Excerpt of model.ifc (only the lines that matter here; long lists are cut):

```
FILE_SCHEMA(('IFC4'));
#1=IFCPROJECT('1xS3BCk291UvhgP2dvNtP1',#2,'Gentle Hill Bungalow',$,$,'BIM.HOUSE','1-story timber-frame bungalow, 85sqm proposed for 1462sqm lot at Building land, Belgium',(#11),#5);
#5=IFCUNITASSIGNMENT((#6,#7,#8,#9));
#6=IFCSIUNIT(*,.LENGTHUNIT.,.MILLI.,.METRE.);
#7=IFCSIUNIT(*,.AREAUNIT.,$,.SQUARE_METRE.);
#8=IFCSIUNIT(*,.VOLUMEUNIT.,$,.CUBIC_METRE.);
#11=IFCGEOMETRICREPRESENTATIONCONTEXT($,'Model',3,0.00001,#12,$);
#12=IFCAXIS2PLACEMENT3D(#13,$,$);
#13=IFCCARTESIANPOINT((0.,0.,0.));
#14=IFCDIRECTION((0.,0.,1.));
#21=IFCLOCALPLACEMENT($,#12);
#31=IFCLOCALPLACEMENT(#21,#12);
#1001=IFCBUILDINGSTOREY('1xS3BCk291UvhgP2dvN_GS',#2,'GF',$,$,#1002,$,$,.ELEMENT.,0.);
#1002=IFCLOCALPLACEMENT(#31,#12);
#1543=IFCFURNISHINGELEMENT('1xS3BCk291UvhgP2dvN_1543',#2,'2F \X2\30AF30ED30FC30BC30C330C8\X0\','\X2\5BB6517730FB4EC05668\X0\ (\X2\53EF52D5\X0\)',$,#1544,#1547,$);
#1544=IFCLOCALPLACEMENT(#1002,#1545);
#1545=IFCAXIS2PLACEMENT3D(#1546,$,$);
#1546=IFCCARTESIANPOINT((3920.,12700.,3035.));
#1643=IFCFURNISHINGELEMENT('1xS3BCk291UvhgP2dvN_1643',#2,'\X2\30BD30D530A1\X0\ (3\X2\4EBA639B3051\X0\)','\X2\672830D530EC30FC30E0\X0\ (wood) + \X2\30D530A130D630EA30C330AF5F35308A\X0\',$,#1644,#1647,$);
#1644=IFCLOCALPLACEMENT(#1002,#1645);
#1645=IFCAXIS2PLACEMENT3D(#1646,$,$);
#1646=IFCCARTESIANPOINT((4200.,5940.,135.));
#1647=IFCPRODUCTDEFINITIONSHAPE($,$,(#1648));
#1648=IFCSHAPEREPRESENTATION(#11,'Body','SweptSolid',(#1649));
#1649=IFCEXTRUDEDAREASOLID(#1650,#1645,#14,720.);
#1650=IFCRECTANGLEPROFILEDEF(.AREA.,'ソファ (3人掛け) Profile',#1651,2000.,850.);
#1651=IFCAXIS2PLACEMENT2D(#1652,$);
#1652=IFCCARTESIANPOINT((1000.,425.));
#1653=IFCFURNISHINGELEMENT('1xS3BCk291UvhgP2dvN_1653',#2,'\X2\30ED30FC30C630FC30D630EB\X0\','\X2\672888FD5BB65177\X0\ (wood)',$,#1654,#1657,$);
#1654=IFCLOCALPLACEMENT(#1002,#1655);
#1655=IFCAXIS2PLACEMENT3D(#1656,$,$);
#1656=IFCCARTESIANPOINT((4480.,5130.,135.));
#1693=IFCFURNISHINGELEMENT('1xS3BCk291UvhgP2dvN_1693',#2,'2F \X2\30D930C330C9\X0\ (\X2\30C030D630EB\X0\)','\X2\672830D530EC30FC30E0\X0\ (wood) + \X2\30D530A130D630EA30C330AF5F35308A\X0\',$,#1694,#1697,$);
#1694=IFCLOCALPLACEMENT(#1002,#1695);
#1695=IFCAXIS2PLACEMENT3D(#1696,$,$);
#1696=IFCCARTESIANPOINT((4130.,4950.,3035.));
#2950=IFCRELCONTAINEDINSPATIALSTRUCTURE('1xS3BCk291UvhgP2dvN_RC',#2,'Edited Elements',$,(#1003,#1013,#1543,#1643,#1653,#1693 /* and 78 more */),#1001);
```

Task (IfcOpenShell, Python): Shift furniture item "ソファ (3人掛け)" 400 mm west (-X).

```python
import ifcopenshell
import ifcopenshell.api.geometry
import ifcopenshell.util.placement

model = ifcopenshell.open("model.ifc")

item = model.by_guid("1xS3BCk291UvhgP2dvN_1643")
matrix = ifcopenshell.util.placement.get_local_placement(item.ObjectPlacement)
matrix[0, 3] -= 400.0
ifcopenshell.api.geometry.edit_object_placement(model, product=item, matrix=matrix, is_si=False)

print(ifcopenshell.util.placement.get_local_placement(item.ObjectPlacement).round(3) + 0.0)

model.write("model_updated.ifc")
```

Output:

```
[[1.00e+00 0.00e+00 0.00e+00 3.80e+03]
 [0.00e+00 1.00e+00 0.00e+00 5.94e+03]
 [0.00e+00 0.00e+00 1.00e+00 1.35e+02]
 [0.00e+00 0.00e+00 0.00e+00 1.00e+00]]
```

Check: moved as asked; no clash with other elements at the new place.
